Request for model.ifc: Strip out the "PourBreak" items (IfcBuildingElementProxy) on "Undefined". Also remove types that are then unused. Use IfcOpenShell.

First a look at what the model holds.

```python
import ifcopenshell
import ifcopenshell.util.element

model = ifcopenshell.open("model.ifc")
print(model.schema)
storey = next(s for s in model.by_type("IfcBuildingStorey") if s.Name == "Undefined")
proxies = [e for e in ifcopenshell.util.element.get_decomposition(storey) if e.is_a("IfcBuildingElementProxy")]
seen = {}
for e in proxies:
    element_type = ifcopenshell.util.element.get_type(e)
    name = element_type.Name if element_type not in (None, e) else None
    seen[name] = seen.get(name, 0) + 1
for name, count in sorted(seen.items(), key=str):
    print(count, "x", name)
```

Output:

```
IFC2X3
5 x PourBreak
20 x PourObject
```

```python
import ifcopenshell
import ifcopenshell.api.root
import ifcopenshell.util.element

model = ifcopenshell.open("model.ifc")

storey = next(s for s in model.by_type("IfcBuildingStorey") if s.Name == "Undefined")
proxies = [e for e in ifcopenshell.util.element.get_decomposition(storey) if e.is_a("IfcBuildingElementProxy")]
targets = [e for e in proxies if (t := ifcopenshell.util.element.get_type(e)) not in (None, e) and t.Name == "PourBreak"]
types = {ifcopenshell.util.element.get_type(e) for e in targets} - {None, *targets}

for e in targets:
    ifcopenshell.api.root.remove_product(model, product=e)
print(len(targets), "removed")

unused = [t for t in types if not ifcopenshell.util.element.get_types(t)]
for t in unused:
    ifcopenshell.api.root.remove_product(model, product=t)
print(len(unused), "unused types removed")

model.write("model_v2.ifc")
```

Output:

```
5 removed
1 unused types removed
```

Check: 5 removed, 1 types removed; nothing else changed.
